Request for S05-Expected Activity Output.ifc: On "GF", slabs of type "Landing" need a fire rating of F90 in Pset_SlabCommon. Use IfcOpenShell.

First a look at what the model holds.

```python
import ifcopenshell
import ifcopenshell.util.element

model = ifcopenshell.open("S05-Expected Activity Output.ifc")
print(model.schema)
storey = next(s for s in model.by_type("IfcBuildingStorey") if s.Name == "GF")
slabs = [e for e in ifcopenshell.util.element.get_decomposition(storey) if e.is_a("IfcSlab")]
seen = {}
for e in slabs:
    element_type = ifcopenshell.util.element.get_type(e)
    key = (element_type.Name if element_type != e and element_type else None, ifcopenshell.util.element.get_pset(e, "Pset_SlabCommon", "FireRating"))
    seen[key] = seen.get(key, 0) + 1
for (name, value), count in sorted(seen.items(), key=str):
    print(count, "x", name, "|", value)
```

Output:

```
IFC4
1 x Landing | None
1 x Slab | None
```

```python
import ifcopenshell
import ifcopenshell.api.pset
import ifcopenshell.util.element

model = ifcopenshell.open("S05-Expected Activity Output.ifc")

storey = next(s for s in model.by_type("IfcBuildingStorey") if s.Name == "GF")
slabs = [e for e in ifcopenshell.util.element.get_decomposition(storey) if e.is_a("IfcSlab")]

count = 0
for e in slabs:
    element_type = ifcopenshell.util.element.get_type(e)
    if element_type in (None, e) or element_type.Name != "Landing":
        continue
    # add_pset returns the element's existing set when there is one.
    pset = ifcopenshell.api.pset.add_pset(model, product=e, name="Pset_SlabCommon")
    ifcopenshell.api.pset.edit_pset(model, pset=pset, properties={"FireRating": "F90"})
    count += 1

print(count, "slabs updated")

model.write("S05-Expected Activity Output_updated.ifc")
```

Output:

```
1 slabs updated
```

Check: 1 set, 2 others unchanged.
